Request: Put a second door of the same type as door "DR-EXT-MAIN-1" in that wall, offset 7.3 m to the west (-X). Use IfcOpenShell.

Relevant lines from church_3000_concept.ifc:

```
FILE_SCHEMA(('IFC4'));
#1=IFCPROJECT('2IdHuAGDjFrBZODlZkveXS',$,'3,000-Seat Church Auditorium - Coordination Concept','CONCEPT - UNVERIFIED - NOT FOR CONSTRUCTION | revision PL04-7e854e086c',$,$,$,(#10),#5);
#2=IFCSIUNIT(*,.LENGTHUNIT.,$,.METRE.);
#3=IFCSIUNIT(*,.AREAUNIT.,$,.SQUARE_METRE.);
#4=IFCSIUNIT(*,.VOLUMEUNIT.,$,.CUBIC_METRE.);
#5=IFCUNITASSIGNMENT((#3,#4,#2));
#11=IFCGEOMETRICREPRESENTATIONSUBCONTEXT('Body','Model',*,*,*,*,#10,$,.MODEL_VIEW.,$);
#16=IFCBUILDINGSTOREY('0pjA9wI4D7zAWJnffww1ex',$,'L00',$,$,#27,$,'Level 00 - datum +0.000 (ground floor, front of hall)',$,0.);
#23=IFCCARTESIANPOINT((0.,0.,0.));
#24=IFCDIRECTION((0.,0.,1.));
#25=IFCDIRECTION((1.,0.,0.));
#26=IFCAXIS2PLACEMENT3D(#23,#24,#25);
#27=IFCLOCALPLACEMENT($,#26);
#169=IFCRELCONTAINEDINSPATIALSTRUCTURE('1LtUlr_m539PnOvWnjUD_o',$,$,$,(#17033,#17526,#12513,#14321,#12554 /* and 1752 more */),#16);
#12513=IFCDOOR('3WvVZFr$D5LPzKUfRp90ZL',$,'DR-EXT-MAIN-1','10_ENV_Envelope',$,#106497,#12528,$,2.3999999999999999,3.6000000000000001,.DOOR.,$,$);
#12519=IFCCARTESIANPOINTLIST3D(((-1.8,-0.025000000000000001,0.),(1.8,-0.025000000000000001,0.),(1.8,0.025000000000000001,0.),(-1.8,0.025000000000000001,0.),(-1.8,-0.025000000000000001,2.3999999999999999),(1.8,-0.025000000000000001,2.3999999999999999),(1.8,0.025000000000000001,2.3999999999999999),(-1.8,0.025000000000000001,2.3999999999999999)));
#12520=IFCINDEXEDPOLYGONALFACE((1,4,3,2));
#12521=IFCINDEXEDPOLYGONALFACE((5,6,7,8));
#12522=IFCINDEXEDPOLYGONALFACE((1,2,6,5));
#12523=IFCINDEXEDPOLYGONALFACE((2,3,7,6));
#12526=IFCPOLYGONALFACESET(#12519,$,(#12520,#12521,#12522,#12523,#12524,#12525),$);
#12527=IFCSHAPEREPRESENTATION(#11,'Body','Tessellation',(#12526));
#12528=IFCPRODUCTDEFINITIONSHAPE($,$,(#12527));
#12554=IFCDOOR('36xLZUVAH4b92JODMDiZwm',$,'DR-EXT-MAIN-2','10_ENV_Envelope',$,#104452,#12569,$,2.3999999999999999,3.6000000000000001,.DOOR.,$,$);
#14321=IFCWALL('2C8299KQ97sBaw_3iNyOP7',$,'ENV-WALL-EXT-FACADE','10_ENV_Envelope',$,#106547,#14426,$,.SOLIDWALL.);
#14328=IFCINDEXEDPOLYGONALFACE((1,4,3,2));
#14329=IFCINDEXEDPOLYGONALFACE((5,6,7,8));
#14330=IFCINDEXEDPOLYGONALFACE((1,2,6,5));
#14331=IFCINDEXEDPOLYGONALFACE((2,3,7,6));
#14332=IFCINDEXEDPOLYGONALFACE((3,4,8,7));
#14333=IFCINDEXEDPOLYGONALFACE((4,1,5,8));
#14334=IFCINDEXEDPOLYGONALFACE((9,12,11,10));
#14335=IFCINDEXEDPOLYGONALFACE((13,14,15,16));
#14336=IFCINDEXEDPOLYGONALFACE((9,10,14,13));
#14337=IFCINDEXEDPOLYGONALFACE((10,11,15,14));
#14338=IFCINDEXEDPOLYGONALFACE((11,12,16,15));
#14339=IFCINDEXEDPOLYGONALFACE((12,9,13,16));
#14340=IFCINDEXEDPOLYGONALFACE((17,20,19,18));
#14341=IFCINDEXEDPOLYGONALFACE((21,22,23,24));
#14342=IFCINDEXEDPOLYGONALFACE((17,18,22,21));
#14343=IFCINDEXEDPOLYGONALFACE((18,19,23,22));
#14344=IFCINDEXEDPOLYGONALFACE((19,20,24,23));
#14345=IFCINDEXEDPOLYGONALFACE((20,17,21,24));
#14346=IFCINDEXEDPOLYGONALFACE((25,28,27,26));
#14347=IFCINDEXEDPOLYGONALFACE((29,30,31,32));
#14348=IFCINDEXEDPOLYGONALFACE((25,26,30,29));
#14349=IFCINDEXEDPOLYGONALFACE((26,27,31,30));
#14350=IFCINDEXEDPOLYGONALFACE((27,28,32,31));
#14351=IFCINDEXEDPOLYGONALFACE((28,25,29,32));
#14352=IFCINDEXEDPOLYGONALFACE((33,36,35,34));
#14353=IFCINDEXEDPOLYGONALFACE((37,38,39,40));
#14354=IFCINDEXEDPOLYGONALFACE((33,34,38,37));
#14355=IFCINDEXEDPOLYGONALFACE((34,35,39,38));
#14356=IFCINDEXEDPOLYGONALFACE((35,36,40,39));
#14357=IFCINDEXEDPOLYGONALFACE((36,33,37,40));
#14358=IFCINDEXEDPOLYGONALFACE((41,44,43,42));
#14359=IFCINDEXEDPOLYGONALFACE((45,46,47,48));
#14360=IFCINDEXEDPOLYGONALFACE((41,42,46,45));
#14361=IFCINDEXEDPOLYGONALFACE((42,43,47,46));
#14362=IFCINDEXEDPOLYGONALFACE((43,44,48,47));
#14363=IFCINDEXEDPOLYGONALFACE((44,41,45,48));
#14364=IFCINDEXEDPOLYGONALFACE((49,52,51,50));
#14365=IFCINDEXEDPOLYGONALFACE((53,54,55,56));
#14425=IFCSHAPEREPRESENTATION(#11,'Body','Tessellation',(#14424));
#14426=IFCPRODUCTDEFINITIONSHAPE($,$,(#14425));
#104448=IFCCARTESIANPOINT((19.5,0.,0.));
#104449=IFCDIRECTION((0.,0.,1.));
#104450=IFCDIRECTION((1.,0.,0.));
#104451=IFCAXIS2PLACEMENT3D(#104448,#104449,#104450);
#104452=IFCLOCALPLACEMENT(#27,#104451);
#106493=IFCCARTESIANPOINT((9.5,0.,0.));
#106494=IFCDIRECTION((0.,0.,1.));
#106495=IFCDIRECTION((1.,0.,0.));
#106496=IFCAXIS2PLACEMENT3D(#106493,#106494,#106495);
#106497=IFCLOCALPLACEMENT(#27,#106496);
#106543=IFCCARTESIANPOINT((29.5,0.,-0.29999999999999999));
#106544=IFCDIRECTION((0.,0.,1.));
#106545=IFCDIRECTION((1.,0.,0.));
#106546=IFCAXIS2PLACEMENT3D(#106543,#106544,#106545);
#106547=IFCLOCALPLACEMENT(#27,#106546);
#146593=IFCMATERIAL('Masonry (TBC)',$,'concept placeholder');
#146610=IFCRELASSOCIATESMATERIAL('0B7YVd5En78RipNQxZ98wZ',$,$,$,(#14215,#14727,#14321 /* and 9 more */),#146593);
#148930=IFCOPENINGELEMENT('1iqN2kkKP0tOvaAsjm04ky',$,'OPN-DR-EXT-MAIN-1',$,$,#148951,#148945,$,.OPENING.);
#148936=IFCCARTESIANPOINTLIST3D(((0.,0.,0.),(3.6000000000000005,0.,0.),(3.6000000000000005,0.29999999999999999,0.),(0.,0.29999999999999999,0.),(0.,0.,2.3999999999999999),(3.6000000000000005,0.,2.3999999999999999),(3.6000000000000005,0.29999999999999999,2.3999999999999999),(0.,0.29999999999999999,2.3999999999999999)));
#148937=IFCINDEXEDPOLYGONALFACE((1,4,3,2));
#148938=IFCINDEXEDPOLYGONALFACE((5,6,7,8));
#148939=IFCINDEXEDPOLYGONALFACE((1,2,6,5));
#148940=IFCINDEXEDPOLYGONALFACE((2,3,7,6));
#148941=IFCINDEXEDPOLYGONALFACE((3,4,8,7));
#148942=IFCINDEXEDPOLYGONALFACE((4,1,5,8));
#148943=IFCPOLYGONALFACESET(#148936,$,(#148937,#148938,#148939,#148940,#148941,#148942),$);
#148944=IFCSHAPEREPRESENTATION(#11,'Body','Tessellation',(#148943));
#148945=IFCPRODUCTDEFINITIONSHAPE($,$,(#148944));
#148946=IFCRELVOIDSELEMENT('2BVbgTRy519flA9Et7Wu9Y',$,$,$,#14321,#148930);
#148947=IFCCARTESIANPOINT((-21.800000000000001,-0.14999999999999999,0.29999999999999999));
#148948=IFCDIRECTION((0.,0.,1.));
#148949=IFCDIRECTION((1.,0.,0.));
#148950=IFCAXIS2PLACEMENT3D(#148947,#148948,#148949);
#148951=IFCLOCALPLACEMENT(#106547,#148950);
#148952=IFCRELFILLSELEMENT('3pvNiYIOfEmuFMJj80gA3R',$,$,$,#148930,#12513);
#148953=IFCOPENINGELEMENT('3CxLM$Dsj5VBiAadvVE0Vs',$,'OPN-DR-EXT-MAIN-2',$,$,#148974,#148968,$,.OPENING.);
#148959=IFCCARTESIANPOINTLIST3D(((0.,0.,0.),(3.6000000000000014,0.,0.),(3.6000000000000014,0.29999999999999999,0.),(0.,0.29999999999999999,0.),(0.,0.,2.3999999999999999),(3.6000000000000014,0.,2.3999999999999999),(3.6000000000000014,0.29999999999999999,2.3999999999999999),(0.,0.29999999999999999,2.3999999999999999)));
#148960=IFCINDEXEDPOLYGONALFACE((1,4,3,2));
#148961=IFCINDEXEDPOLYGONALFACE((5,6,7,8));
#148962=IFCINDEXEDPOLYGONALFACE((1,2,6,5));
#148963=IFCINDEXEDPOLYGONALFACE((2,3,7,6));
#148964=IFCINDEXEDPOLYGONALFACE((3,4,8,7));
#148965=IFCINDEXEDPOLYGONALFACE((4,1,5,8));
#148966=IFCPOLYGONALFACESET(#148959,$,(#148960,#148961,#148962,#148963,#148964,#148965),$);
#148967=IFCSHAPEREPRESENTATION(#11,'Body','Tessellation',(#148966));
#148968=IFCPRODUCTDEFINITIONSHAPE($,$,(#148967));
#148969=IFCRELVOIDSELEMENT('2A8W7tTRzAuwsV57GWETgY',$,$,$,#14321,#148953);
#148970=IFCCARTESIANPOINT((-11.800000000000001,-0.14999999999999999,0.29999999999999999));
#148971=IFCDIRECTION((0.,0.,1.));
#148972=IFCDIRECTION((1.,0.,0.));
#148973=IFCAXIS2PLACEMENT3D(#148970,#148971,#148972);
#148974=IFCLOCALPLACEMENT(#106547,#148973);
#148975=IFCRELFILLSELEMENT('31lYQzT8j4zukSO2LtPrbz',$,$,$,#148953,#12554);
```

```python
import ifcopenshell
import ifcopenshell.api.feature
import ifcopenshell.api.geometry
import ifcopenshell.api.root
import ifcopenshell.geom
import ifcopenshell.util.element
import ifcopenshell.util.placement
import ifcopenshell.util.shape
import ifcopenshell.util.unit

model = ifcopenshell.open("church_3000_concept.ifc")
unit_scale = ifcopenshell.util.unit.calculate_unit_scale(model)
settings = ifcopenshell.geom.settings()


def volume(element):
    """Net volume in cubic metres, openings subtracted."""
    shape = ifcopenshell.geom.create_shape(settings, element)
    return ifcopenshell.util.shape.get_volume(shape.geometry)


door = model.by_guid("3WvVZFr$D5LPzKUfRp90ZL")
opening = door.FillsVoids[0].RelatingOpeningElement
wall = opening.VoidsElements[0].RelatingBuildingElement
before = volume(wall)
shift = ifcopenshell.util.placement.get_local_placement(wall.ObjectPlacement)[:3, 0] * -7.3 / unit_scale

# copy_class copies the void relationship, type, container and properties, but no geometry.
new_opening = ifcopenshell.api.root.copy_class(model, product=opening)
new_opening.Representation = ifcopenshell.util.element.copy_deep(
    model, opening.Representation, exclude=["IfcGeometricRepresentationContext", "IfcRepresentationMap"]
)
new_door = ifcopenshell.api.root.copy_class(model, product=door)
new_door.Representation = ifcopenshell.util.element.copy_deep(
    model, door.Representation, exclude=["IfcGeometricRepresentationContext", "IfcRepresentationMap"]
)
ifcopenshell.api.feature.add_filling(model, opening=new_opening, element=new_door)

for old, new in ((opening, new_opening), (door, new_door)):
    matrix = ifcopenshell.util.placement.get_local_placement(old.ObjectPlacement)
    matrix[:3, 3] += shift
    ifcopenshell.api.geometry.edit_object_placement(model, product=new, matrix=matrix, is_si=False)

after = volume(wall)

print(f"wall volume {before:.3f} -> {after:.3f} m3")

model.write("church_3000_concept_rev.ifc")
```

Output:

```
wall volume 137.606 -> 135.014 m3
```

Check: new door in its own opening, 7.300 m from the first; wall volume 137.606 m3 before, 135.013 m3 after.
